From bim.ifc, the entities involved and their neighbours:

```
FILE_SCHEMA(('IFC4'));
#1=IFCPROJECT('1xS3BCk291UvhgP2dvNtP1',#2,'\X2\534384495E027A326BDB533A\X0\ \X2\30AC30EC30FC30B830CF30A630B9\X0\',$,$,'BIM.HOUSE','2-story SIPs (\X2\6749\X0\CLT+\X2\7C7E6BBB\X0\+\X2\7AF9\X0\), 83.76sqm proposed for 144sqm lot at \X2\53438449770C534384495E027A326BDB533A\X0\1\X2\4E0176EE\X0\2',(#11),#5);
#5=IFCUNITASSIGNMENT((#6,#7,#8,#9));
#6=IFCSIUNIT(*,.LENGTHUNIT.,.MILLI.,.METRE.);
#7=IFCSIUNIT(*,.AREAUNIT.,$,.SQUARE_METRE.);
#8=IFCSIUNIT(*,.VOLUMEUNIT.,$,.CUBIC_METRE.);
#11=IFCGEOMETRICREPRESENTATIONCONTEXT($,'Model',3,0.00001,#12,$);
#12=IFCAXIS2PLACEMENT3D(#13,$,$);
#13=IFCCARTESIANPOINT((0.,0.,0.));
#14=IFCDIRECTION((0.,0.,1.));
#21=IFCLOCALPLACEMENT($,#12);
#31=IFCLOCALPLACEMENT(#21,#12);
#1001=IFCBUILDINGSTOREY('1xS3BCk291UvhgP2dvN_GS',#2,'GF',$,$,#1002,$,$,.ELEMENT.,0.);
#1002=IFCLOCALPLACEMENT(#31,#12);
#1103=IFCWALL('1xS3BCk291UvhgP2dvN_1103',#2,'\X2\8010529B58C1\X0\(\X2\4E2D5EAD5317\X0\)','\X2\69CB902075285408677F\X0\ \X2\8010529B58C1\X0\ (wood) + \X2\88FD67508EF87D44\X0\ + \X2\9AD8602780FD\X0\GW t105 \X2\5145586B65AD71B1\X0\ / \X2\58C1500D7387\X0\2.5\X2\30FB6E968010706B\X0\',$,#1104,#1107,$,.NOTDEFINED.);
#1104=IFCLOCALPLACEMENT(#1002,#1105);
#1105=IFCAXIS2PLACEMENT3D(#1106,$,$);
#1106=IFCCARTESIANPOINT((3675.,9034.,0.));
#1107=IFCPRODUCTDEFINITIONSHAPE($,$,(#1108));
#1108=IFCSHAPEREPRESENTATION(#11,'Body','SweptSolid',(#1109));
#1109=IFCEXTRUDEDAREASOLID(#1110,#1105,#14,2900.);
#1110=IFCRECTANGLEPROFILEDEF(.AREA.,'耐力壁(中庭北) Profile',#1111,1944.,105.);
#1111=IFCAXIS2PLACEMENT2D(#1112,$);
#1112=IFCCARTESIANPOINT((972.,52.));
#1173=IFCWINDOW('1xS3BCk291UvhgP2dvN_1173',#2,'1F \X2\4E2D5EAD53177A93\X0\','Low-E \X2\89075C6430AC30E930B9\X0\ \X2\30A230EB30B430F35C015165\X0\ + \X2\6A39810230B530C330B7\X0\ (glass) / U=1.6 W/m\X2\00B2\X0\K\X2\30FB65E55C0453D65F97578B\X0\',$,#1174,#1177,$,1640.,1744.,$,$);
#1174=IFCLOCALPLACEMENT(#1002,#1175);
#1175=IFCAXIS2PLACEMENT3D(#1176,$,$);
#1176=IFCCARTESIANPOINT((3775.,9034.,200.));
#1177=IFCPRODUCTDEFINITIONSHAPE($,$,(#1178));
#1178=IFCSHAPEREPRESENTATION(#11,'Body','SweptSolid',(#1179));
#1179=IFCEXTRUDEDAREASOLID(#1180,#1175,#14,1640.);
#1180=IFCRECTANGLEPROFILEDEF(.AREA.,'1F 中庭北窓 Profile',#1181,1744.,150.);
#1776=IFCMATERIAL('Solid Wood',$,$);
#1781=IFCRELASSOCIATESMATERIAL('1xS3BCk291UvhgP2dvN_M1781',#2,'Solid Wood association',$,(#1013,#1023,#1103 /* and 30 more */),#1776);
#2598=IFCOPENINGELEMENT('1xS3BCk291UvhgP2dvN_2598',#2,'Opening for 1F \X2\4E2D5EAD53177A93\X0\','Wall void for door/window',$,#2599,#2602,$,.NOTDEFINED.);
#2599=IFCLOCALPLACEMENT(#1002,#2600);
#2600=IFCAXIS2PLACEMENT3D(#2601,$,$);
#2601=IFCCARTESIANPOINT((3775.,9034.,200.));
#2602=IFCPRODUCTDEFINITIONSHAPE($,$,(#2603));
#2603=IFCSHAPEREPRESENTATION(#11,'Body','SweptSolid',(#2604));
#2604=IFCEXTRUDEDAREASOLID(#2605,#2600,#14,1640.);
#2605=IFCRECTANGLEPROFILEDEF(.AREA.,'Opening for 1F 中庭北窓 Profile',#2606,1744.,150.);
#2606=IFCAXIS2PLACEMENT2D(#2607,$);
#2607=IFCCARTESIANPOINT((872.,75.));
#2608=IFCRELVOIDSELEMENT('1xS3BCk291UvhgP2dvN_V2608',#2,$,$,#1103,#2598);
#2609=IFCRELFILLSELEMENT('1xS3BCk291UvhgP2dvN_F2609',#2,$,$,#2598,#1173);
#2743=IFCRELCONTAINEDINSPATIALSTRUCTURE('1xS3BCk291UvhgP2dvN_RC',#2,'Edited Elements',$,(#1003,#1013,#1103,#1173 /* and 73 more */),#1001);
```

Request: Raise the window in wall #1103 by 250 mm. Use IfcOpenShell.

```python
import numpy as np
import ifcopenshell
import ifcopenshell.api.geometry
import ifcopenshell.util.placement
import ifcopenshell.util.unit

model = ifcopenshell.open("bim.ifc")
unit_scale = ifcopenshell.util.unit.calculate_unit_scale(model)

window = model.by_guid("1xS3BCk291UvhgP2dvN_1173")
opening = window.FillsVoids[0].RelatingOpeningElement
dz = 250.0

shift = np.array([0.0, 0.0, dz])
# The window is not placed relative to its opening, so move both.
for product in (opening, window):
    matrix = ifcopenshell.util.placement.get_local_placement(product.ObjectPlacement)
    matrix[:3, 3] += shift
    ifcopenshell.api.geometry.edit_object_placement(model, product=product, matrix=matrix, is_si=False)

print(f"moved by {dz * unit_scale:+.3f} m")

model.write("bim_updated.ifc")
```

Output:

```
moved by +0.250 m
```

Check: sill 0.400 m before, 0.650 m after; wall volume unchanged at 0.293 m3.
